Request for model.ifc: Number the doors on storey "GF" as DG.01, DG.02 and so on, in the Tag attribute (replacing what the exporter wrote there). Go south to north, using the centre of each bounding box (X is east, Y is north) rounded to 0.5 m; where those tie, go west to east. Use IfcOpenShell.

First a look at what the model holds.

```python
import ifcopenshell
import ifcopenshell.util.element
import ifcopenshell.util.placement

model = ifcopenshell.open("model.ifc")
print(model.schema)
storey = next(s for s in model.by_type("IfcBuildingStorey") if s.Name == "GF")
doors = [e for e in ifcopenshell.util.element.get_decomposition(storey) if e.is_a("IfcDoor")]
for e in sorted(doors, key=lambda e: e.id()):
    origin = ifcopenshell.util.placement.get_local_placement(e.ObjectPlacement)[:3, 3]
    print(e.id(), e.Tag, e.Name, origin.round(2) + 0.0, sep=" | ")
```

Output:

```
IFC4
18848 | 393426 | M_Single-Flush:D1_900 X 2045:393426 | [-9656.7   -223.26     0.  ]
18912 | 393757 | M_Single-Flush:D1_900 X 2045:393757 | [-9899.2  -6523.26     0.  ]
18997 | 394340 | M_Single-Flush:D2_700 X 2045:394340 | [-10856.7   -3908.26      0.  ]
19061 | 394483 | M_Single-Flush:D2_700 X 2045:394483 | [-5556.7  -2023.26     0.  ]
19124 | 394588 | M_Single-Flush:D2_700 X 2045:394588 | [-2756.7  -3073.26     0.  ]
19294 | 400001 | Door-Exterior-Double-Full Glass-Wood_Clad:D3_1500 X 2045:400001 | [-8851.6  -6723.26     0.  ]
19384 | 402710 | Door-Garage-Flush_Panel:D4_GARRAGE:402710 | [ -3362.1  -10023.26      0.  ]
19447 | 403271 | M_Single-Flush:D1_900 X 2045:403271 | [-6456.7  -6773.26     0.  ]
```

```python
import ifcopenshell
import ifcopenshell.geom
import ifcopenshell.util.element
import ifcopenshell.util.shape

model = ifcopenshell.open("model.ifc")
settings = ifcopenshell.geom.settings()
settings.set("use-world-coords", True)


def centre(element):
    shape = ifcopenshell.geom.create_shape(settings, element)
    return ifcopenshell.util.shape.get_bbox_centroid(shape.geometry)


storey = next(s for s in model.by_type("IfcBuildingStorey") if s.Name == "GF")
doors = [e for e in ifcopenshell.util.element.get_decomposition(storey) if e.is_a("IfcDoor")]

# Insertion points can sit at a corner or the storey origin, so sort by the geometry (in metres).
centres = {e: centre(e) for e in doors}
doors.sort(key=lambda e: (round(centres[e][1] / 0.5), centres[e][0]))

for i, e in enumerate(doors, start=1):
    number = f"DG.{i:02d}"
    e.Tag = number
    print(e.id(), number)

model.write("model_rev.ifc")
```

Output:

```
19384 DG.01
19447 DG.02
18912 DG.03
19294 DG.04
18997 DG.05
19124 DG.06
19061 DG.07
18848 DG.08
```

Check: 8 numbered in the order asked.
